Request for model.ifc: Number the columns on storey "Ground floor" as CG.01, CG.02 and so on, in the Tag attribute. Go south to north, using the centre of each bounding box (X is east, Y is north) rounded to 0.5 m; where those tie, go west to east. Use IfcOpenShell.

First a look at what the model holds.

```python
import ifcopenshell
import ifcopenshell.util.element
import ifcopenshell.util.placement

model = ifcopenshell.open("model.ifc")
print(model.schema)
storey = next(s for s in model.by_type("IfcBuildingStorey") if s.Name == "Ground floor")
columns = [e for e in ifcopenshell.util.element.get_decomposition(storey) if e.is_a("IfcColumn")]
for e in sorted(columns, key=lambda e: e.id()):
    origin = ifcopenshell.util.placement.get_local_placement(e.ObjectPlacement)[:3, 3]
    print(e.id(), e.Tag, e.Name, origin.round(2) + 0.0, sep=" | ")
```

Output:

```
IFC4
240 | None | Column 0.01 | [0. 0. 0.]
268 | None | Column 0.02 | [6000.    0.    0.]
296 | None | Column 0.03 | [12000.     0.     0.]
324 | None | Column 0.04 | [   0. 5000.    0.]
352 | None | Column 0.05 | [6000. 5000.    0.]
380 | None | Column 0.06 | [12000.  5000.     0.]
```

```python
import ifcopenshell
import ifcopenshell.geom
import ifcopenshell.util.element
import ifcopenshell.util.shape

model = ifcopenshell.open("model.ifc")
settings = ifcopenshell.geom.settings()
settings.set("use-world-coords", True)


def centre(element):
    shape = ifcopenshell.geom.create_shape(settings, element)
    return ifcopenshell.util.shape.get_bbox_centroid(shape.geometry)


storey = next(s for s in model.by_type("IfcBuildingStorey") if s.Name == "Ground floor")
columns = [e for e in ifcopenshell.util.element.get_decomposition(storey) if e.is_a("IfcColumn")]

# Insertion points can sit at a corner or the storey origin, so sort by the geometry (in metres).
centres = {e: centre(e) for e in columns}
columns.sort(key=lambda e: (round(centres[e][1] / 0.5), centres[e][0]))

for i, e in enumerate(columns, start=1):
    number = f"CG.{i:02d}"
    e.Tag = number
    print(e.id(), number)

model.write("model-out.ifc")
```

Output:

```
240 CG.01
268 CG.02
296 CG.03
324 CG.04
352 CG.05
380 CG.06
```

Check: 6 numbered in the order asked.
